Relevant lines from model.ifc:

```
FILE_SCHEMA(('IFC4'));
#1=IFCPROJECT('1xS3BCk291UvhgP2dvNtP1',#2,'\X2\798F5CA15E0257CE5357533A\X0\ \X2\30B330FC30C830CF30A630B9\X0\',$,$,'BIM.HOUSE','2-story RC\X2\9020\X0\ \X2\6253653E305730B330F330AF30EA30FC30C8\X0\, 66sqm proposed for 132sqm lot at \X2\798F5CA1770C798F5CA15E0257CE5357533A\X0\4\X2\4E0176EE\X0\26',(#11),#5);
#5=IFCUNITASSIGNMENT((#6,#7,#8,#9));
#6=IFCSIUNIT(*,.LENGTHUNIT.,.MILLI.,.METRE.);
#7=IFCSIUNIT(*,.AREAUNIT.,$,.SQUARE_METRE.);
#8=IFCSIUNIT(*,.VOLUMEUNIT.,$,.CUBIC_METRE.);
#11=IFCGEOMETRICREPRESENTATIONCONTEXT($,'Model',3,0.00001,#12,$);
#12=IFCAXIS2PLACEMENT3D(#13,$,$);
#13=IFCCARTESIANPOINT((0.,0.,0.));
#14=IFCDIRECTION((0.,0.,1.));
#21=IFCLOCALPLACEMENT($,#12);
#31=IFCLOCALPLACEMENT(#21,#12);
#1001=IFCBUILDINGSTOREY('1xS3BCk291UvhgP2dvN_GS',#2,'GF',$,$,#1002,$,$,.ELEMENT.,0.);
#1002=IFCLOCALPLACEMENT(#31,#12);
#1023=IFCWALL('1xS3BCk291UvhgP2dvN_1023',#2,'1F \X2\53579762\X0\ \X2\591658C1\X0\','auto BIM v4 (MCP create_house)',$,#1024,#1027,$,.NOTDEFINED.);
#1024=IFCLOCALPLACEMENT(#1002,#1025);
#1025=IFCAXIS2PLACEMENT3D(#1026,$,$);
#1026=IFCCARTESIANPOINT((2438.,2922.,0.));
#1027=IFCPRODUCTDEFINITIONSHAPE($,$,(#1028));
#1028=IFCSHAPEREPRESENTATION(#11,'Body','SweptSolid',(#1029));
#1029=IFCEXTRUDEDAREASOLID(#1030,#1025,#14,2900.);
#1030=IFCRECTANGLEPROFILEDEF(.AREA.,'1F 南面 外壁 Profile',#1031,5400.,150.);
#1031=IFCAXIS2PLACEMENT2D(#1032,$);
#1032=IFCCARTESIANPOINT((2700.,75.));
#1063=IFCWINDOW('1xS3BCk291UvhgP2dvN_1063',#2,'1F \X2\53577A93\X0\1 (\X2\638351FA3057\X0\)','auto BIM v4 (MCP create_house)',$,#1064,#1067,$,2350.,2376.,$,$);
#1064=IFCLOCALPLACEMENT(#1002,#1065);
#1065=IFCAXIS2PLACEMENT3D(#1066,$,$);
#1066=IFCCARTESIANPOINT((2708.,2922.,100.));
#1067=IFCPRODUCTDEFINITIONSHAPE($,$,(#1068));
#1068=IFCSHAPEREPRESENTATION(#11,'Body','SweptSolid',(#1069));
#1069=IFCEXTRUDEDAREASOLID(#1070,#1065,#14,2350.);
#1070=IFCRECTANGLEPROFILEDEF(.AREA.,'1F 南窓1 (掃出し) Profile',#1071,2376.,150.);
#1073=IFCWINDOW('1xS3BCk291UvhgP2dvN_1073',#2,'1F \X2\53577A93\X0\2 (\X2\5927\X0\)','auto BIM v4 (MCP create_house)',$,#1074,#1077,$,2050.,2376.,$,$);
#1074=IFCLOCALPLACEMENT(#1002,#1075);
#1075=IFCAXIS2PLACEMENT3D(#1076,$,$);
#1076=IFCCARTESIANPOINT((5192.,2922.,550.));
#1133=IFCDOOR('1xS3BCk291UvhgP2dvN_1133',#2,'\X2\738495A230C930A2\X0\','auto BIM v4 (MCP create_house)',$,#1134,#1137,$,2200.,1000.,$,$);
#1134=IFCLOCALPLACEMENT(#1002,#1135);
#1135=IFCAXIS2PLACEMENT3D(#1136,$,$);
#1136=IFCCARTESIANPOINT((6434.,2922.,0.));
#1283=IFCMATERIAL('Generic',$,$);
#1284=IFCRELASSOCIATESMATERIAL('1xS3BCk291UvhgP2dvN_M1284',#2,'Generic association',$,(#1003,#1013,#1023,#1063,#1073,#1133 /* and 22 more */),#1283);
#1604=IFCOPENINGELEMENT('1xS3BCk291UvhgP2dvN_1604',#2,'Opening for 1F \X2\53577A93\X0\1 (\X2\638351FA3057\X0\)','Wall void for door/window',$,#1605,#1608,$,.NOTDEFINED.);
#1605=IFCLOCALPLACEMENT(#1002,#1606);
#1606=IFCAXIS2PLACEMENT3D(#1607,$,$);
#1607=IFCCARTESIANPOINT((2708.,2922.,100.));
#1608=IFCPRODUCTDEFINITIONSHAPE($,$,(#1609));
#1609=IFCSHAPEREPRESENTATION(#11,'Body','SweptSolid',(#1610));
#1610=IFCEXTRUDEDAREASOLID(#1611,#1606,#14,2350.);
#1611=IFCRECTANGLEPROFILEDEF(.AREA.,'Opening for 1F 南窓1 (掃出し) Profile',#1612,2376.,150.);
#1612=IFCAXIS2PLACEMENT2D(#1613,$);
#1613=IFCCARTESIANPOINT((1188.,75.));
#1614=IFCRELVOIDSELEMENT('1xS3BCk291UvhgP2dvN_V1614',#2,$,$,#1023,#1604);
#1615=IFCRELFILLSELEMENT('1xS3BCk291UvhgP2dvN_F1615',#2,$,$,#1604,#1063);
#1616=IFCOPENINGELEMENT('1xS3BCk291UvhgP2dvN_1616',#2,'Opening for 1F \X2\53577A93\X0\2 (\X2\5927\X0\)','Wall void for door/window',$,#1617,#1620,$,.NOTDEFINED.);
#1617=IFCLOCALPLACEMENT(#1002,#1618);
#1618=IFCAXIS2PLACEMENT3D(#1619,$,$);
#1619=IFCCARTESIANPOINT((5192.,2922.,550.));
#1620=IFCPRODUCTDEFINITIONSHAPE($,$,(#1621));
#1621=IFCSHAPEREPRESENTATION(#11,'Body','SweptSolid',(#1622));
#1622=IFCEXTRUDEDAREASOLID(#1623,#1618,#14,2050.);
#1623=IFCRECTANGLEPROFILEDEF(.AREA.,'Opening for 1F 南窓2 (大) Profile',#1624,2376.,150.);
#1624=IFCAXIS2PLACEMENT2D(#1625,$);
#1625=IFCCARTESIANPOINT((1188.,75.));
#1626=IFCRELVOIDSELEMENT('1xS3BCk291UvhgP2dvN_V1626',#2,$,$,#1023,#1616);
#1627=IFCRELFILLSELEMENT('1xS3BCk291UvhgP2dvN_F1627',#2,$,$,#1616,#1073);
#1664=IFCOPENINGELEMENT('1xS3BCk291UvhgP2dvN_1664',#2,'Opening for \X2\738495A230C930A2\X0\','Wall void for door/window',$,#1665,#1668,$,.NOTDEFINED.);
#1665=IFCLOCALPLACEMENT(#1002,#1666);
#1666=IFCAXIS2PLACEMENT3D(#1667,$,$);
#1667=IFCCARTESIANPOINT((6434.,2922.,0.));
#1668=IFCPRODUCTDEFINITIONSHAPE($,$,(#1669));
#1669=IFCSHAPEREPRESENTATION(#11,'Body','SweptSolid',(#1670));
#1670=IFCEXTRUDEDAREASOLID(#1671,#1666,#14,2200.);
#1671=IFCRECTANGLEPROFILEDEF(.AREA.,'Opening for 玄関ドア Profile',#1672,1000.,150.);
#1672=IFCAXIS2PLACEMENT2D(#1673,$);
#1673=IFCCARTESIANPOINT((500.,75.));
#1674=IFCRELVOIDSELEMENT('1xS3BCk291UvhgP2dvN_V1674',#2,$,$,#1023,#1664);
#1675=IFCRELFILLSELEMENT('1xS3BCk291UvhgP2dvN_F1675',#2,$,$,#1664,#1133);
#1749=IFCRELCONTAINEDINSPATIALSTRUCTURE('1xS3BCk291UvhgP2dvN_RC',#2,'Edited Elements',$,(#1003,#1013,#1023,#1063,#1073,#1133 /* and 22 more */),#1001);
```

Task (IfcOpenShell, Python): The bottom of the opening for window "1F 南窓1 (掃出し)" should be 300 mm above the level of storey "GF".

```python
import numpy as np
import ifcopenshell
import ifcopenshell.api.geometry
import ifcopenshell.geom
import ifcopenshell.util.element
import ifcopenshell.util.placement
import ifcopenshell.util.shape
import ifcopenshell.util.unit

model = ifcopenshell.open("model.ifc")
unit_scale = ifcopenshell.util.unit.calculate_unit_scale(model)

window = model.by_guid("1xS3BCk291UvhgP2dvN_1063")
opening = window.FillsVoids[0].RelatingOpeningElement
storey = ifcopenshell.util.element.get_container(window, ifc_class="IfcBuildingStorey")
level = ifcopenshell.util.placement.get_local_placement(storey.ObjectPlacement)[2, 3]

# The opening's origin need not be at the sill, so measure its lowest point.
shape = ifcopenshell.geom.create_shape(ifcopenshell.geom.settings(), opening)
bottom = ifcopenshell.util.shape.get_shape_bottom_elevation(shape, shape.geometry) / unit_scale
dz = level + 0.3 / unit_scale - bottom

shift = np.array([0.0, 0.0, dz])
# The window is not placed relative to its opening, so move both.
for product in (opening, window):
    matrix = ifcopenshell.util.placement.get_local_placement(product.ObjectPlacement)
    matrix[:3, 3] += shift
    ifcopenshell.api.geometry.edit_object_placement(model, product=product, matrix=matrix, is_si=False)

print(f"moved by {dz * unit_scale:+.3f} m")

model.write("model-out.ifc")
```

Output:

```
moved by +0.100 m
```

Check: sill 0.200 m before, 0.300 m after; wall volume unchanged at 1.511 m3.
